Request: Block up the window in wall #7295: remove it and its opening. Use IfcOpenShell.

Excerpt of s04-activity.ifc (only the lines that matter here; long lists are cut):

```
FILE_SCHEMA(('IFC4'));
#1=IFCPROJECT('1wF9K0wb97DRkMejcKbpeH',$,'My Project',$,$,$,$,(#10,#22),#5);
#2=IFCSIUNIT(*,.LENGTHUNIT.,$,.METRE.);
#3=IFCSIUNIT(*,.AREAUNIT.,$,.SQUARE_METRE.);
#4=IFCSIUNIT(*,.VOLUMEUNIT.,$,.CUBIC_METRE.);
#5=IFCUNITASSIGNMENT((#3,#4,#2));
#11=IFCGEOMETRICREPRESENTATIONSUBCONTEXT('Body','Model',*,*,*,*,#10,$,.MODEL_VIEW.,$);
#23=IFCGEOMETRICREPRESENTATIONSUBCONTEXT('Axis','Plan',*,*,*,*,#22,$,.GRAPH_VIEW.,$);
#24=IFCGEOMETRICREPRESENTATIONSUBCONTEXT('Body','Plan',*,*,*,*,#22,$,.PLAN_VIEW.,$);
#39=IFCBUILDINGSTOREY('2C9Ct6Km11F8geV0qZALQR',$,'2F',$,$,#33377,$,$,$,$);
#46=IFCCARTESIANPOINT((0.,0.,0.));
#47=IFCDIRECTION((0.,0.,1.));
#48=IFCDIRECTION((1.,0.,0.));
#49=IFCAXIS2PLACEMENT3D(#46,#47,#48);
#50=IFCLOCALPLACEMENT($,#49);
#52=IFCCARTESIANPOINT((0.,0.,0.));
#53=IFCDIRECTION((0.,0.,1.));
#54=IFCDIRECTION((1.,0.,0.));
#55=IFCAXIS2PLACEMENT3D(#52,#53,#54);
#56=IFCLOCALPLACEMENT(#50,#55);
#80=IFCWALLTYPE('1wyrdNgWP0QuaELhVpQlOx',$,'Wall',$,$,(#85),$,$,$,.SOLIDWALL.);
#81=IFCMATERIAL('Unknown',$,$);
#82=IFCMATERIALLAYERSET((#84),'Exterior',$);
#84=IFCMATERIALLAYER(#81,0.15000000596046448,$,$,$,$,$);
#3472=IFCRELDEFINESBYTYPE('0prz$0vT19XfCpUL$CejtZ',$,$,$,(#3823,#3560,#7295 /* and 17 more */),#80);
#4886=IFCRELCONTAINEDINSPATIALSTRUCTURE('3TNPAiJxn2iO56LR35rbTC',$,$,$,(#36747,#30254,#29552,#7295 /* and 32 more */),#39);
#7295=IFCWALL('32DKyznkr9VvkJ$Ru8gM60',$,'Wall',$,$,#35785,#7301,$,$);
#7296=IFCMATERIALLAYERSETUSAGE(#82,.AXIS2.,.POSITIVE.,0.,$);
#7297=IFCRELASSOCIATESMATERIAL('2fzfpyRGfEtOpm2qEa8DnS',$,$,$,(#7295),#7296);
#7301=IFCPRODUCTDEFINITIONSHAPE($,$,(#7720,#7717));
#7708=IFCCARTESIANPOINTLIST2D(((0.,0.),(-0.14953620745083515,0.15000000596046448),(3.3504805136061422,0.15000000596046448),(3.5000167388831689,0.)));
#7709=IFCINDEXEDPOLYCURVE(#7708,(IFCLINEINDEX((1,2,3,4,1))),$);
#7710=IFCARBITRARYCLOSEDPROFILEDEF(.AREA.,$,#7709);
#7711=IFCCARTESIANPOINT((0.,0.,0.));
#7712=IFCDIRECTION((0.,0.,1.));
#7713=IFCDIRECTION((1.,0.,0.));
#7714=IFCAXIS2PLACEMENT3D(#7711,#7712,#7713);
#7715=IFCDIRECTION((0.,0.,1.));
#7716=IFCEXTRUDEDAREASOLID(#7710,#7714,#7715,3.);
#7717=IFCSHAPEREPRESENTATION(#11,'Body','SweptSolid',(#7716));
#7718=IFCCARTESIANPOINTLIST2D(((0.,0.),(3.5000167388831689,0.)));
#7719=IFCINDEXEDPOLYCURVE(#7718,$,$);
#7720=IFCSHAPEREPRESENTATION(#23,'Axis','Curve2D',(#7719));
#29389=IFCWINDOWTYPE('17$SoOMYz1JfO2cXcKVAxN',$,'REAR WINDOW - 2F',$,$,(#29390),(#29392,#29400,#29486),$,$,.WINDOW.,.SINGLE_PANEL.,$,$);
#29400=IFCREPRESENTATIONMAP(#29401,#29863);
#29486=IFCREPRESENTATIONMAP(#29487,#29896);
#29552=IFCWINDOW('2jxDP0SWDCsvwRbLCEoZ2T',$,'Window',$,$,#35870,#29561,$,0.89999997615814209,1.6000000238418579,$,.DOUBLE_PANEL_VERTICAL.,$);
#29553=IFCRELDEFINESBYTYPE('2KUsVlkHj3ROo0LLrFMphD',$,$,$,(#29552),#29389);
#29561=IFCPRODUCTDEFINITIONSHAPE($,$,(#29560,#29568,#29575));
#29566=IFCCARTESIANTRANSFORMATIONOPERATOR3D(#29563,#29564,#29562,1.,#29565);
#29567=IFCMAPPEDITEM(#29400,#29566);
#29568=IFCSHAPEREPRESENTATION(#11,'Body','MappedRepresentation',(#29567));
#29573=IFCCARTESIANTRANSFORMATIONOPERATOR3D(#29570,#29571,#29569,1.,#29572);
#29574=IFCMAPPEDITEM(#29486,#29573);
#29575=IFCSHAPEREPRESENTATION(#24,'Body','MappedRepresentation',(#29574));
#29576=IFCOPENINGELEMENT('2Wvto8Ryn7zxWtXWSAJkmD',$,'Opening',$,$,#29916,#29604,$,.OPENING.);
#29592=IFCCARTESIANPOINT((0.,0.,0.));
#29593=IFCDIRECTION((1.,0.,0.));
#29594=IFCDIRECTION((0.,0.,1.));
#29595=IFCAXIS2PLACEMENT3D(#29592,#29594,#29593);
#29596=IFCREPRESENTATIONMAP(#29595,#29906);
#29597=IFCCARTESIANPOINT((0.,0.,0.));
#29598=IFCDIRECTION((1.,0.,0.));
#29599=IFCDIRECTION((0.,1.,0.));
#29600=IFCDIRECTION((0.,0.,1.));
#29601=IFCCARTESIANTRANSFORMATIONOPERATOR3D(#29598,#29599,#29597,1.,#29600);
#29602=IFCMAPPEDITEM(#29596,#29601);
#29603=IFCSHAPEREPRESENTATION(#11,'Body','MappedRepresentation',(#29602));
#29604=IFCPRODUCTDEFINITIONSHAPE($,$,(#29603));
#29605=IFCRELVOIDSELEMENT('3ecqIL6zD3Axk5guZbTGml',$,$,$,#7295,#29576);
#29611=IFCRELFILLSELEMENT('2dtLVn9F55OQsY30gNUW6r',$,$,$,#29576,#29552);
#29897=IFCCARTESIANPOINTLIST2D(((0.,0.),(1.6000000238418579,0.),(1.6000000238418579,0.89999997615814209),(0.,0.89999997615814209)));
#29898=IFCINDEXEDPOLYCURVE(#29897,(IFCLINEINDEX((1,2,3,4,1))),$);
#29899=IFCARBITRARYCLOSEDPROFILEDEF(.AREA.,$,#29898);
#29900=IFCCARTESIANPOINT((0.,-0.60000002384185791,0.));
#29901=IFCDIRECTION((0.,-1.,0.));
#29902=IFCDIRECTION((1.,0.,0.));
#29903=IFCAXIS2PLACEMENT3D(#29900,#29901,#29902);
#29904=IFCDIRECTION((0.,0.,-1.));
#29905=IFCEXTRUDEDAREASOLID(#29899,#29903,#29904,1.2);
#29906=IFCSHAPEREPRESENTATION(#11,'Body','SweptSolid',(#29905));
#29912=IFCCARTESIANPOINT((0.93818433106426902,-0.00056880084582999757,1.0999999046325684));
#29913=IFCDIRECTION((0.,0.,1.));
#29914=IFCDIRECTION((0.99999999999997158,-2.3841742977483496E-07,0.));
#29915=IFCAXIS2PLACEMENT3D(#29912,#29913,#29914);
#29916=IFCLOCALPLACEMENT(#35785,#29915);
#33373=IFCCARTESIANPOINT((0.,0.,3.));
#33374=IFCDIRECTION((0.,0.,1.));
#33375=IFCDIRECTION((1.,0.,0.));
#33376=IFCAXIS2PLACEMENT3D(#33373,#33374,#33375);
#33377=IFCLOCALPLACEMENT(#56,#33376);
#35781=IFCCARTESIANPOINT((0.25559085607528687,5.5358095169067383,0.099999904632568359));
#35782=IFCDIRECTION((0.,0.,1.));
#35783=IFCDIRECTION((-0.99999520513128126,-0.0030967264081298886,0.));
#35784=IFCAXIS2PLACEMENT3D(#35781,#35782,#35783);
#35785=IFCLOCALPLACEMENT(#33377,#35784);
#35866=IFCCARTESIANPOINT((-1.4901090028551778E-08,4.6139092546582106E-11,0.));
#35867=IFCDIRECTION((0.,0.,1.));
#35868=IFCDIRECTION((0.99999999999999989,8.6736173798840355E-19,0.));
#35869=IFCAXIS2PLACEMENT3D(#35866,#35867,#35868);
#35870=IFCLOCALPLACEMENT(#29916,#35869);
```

```python
import ifcopenshell
import ifcopenshell.api.feature
import ifcopenshell.api.root
import ifcopenshell.geom
import ifcopenshell.util.shape

model = ifcopenshell.open("s04-activity.ifc")
settings = ifcopenshell.geom.settings()


def volume(element):
    """Net volume in cubic metres, openings subtracted."""
    shape = ifcopenshell.geom.create_shape(settings, element)
    return ifcopenshell.util.shape.get_volume(shape.geometry)


window = model.by_guid("2jxDP0SWDCsvwRbLCEoZ2T")
opening = window.FillsVoids[0].RelatingOpeningElement
wall = opening.VoidsElements[0].RelatingBuildingElement
before = volume(wall)

ifcopenshell.api.root.remove_product(model, product=window)
ifcopenshell.api.feature.remove_feature(model, feature=opening)

after = volume(wall)

print(f"wall volume {before:.3f} -> {after:.3f} m3")

model.write("s04-activity_updated.ifc")
```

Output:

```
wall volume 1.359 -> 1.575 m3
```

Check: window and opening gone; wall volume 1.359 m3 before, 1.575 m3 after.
